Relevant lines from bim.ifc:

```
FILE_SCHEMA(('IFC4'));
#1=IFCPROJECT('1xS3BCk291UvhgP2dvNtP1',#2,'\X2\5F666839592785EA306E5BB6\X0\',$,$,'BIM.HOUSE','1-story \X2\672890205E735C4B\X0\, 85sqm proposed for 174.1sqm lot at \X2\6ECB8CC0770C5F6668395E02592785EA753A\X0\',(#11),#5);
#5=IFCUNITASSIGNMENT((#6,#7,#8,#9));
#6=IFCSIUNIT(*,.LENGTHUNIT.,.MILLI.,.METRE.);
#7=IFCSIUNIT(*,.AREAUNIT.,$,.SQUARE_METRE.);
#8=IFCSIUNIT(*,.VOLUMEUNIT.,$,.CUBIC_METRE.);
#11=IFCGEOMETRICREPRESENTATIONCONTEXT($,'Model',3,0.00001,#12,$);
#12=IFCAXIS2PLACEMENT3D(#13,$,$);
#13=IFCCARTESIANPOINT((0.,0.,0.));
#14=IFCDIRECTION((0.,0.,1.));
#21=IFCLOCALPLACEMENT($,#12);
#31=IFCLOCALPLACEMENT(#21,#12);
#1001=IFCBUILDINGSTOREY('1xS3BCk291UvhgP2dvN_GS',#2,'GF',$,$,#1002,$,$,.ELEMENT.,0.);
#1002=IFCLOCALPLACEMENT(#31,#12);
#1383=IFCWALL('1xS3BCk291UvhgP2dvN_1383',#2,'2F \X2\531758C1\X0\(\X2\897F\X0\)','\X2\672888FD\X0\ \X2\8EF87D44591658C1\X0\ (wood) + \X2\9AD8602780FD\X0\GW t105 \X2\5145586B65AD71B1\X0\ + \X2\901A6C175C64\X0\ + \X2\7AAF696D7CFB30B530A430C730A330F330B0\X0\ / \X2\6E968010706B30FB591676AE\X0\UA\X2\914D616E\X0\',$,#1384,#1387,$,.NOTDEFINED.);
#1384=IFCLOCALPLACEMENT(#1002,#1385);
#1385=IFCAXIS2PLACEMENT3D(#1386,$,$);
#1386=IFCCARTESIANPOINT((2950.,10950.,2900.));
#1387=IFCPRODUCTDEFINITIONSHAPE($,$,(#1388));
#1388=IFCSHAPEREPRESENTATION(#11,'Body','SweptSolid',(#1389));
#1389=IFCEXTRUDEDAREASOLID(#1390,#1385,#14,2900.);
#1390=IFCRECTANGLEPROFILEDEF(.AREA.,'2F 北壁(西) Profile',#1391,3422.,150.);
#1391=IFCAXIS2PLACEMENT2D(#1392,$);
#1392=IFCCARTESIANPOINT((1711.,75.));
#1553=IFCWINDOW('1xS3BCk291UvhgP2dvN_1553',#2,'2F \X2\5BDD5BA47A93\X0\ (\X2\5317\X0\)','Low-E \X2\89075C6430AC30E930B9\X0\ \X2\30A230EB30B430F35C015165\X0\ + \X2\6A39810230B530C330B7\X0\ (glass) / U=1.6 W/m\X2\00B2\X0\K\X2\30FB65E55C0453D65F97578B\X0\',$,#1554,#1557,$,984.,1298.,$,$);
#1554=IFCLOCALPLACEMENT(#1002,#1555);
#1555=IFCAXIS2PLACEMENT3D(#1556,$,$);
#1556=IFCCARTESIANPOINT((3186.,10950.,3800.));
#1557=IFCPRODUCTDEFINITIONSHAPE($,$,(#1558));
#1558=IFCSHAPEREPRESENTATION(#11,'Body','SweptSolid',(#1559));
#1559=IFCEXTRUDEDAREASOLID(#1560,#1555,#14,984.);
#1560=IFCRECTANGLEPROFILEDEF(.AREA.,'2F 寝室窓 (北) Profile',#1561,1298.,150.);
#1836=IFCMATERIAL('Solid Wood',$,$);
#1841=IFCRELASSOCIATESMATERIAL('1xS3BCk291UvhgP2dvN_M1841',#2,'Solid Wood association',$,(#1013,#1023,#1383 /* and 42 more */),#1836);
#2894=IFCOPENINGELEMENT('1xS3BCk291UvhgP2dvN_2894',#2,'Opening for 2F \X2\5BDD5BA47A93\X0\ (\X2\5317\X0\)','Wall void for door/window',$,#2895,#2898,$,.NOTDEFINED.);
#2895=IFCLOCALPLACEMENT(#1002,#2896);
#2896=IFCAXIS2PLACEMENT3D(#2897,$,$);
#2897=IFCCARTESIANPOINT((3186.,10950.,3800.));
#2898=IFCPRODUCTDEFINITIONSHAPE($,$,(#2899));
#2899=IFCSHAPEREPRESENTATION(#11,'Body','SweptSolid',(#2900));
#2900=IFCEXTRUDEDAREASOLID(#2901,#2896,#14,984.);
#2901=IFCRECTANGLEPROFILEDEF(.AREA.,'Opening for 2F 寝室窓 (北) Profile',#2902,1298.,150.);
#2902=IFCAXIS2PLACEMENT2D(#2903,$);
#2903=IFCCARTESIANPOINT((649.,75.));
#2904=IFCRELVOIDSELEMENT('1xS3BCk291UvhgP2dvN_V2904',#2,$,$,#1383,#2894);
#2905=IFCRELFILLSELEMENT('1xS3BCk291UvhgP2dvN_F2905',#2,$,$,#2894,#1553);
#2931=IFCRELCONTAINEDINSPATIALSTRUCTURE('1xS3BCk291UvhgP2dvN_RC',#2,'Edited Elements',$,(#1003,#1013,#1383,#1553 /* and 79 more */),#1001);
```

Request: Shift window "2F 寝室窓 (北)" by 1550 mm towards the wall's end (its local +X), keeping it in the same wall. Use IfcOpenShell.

```python
import ifcopenshell
import ifcopenshell.api.geometry
import ifcopenshell.util.placement
import ifcopenshell.util.unit

model = ifcopenshell.open("bim.ifc")
unit_scale = ifcopenshell.util.unit.calculate_unit_scale(model)

window = model.by_guid("1xS3BCk291UvhgP2dvN_1553")
opening = window.FillsVoids[0].RelatingOpeningElement
wall = opening.VoidsElements[0].RelatingBuildingElement

wall_matrix = ifcopenshell.util.placement.get_local_placement(wall.ObjectPlacement)
shift = wall_matrix[:3, 0] * 1.55 / unit_scale
before = ifcopenshell.util.placement.get_local_placement(window.ObjectPlacement)[:3, 3].copy()

# The window is not placed relative to its opening, so move both.
for product in (opening, window):
    matrix = ifcopenshell.util.placement.get_local_placement(product.ObjectPlacement)
    matrix[:3, 3] += shift
    ifcopenshell.api.geometry.edit_object_placement(model, product=product, matrix=matrix, is_si=False)

after = ifcopenshell.util.placement.get_local_placement(window.ObjectPlacement)[:3, 3]
print("window moved by", (after - before).round(3) + 0.0)

model.write("bim-out.ifc")
```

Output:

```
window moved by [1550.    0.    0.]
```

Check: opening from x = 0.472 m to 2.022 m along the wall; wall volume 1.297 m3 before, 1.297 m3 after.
